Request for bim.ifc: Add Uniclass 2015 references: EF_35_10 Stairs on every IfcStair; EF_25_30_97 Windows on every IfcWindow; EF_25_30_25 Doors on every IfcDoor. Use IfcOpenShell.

First a look at what the model holds.

```python
import ifcopenshell

model = ifcopenshell.open("bim.ifc")
print(model.schema)
print("classifications:", [c.Name for c in model.by_type("IfcClassification")])
for ifc_class in ("IfcDoor", "IfcRoof", "IfcStair", "IfcWall", "IfcWindow"):
    print(ifc_class, len(model.by_type(ifc_class)))
```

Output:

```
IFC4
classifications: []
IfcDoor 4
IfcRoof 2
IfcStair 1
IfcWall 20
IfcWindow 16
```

```python
import ifcopenshell
import ifcopenshell.api.classification

model = ifcopenshell.open("bim.ifc")

system = ifcopenshell.api.classification.add_classification(model, classification="Uniclass 2015")

codes = {
    "IfcStair": ("EF_35_10", "Stairs"),
    "IfcWindow": ("EF_25_30_97", "Windows"),
    "IfcDoor": ("EF_25_30_25", "Doors"),
}
for ifc_class, (code, name) in codes.items():
    products = model.by_type(ifc_class)
    ifcopenshell.api.classification.add_reference(
        model, products=products, classification=system, identification=code, name=name
    )
    print(code, len(products))

model.write("bim_v2.ifc")
```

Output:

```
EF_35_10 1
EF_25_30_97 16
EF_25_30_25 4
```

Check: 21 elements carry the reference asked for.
